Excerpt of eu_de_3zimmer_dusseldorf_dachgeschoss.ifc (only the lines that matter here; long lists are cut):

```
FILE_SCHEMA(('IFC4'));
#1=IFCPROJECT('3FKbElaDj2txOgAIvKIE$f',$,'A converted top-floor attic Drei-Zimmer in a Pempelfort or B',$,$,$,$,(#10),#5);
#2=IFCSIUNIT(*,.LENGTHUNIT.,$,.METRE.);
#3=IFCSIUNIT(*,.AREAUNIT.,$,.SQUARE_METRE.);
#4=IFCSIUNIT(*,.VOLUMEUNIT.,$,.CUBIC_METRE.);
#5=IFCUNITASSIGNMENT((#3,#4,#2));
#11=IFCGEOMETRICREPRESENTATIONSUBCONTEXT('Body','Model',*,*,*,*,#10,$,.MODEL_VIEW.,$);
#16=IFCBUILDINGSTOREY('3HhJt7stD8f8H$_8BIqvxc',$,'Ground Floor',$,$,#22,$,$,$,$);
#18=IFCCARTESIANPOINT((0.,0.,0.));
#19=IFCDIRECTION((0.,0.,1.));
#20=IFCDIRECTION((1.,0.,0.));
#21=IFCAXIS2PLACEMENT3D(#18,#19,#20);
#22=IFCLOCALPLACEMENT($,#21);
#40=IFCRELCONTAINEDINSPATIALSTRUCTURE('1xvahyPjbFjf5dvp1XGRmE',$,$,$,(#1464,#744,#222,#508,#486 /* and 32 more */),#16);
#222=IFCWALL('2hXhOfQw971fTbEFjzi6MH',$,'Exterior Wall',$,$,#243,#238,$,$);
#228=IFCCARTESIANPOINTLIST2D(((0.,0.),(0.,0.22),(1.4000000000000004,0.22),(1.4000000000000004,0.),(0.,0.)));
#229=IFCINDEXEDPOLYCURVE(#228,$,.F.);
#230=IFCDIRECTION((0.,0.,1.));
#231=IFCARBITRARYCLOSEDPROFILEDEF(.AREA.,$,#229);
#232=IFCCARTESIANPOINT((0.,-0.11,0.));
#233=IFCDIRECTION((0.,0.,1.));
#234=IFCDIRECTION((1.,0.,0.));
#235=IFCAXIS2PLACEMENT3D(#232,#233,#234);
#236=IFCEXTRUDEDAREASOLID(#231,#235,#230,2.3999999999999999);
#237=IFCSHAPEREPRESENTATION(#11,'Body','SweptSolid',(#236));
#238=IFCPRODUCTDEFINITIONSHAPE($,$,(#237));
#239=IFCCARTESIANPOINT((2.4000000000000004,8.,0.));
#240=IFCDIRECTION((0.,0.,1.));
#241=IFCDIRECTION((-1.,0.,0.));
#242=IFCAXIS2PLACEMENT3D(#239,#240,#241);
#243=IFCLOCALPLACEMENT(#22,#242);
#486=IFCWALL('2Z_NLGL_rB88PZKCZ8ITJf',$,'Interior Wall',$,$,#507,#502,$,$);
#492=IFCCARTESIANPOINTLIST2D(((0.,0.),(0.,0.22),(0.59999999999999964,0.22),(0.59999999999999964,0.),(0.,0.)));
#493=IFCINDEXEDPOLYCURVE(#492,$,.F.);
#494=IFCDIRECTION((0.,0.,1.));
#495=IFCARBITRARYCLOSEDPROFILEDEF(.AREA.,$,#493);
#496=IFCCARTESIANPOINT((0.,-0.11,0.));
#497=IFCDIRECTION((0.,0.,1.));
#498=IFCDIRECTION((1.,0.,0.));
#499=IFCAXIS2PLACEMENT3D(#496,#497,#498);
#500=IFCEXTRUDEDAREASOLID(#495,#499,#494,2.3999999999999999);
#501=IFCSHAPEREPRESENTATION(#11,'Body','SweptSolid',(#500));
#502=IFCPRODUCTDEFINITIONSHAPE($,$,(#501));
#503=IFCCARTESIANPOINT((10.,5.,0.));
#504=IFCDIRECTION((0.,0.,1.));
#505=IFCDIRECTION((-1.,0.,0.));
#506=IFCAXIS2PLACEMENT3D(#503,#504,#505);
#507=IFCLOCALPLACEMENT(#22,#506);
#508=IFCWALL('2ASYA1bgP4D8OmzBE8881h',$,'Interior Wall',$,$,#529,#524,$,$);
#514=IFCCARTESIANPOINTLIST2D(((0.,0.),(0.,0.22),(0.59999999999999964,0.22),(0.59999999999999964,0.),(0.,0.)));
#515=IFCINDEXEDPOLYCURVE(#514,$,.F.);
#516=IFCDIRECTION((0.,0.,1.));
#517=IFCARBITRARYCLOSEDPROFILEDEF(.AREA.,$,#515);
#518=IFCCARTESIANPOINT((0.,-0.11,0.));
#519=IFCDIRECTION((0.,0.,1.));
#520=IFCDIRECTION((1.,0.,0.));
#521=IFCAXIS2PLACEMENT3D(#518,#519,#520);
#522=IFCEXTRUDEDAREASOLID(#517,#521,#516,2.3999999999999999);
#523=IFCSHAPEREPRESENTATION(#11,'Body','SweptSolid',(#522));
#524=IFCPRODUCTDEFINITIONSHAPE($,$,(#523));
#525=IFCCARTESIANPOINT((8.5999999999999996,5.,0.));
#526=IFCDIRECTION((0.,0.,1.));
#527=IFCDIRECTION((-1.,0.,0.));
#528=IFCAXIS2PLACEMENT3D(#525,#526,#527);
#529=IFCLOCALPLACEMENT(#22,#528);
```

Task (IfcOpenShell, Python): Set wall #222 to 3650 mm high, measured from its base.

```python
import ifcopenshell
import ifcopenshell.geom
import ifcopenshell.util.representation
import ifcopenshell.util.shape

model = ifcopenshell.open("eu_de_3zimmer_dusseldorf_dachgeschoss.ifc")
settings = ifcopenshell.geom.settings()


def volume(element):
    """Net volume in cubic metres, openings subtracted."""
    shape = ifcopenshell.geom.create_shape(settings, element)
    return ifcopenshell.util.shape.get_volume(shape.geometry)


wall = model.by_guid("2hXhOfQw971fTbEFjzi6MH")
before = volume(wall)

body = ifcopenshell.util.representation.get_representation(wall, "Model", "Body")
solid = body.Items[0]
old_height = solid.Depth
solid.Depth = 3.65
after = volume(wall)

print(f"height {old_height:g} -> {solid.Depth:g}, volume {before:.3f} -> {after:.3f} m3")

model.write("eu_de_3zimmer_dusseldorf_dachgeschoss_updated.ifc")
```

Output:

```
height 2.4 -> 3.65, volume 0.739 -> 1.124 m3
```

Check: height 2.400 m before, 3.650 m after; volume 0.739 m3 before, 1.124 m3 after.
